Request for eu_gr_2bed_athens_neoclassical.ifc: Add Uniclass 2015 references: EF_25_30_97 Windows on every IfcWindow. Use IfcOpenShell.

First a look at what the model holds.

```python
import ifcopenshell

model = ifcopenshell.open("eu_gr_2bed_athens_neoclassical.ifc")
print(model.schema)
print("classifications:", [c.Name for c in model.by_type("IfcClassification")])
for ifc_class in ("IfcDoor", "IfcRoof", "IfcStair", "IfcWall", "IfcWindow"):
    print(ifc_class, len(model.by_type(ifc_class)))
```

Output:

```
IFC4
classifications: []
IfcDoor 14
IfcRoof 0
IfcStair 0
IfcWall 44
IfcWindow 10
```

```python
import ifcopenshell
import ifcopenshell.api.classification

model = ifcopenshell.open("eu_gr_2bed_athens_neoclassical.ifc")

system = ifcopenshell.api.classification.add_classification(model, classification="Uniclass 2015")

codes = {
    "IfcWindow": ("EF_25_30_97", "Windows"),
}
for ifc_class, (code, name) in codes.items():
    products = model.by_type(ifc_class)
    ifcopenshell.api.classification.add_reference(
        model, products=products, classification=system, identification=code, name=name
    )
    print(code, len(products))

model.write("eu_gr_2bed_athens_neoclassical-out.ifc")
```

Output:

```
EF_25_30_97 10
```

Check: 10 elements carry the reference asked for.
